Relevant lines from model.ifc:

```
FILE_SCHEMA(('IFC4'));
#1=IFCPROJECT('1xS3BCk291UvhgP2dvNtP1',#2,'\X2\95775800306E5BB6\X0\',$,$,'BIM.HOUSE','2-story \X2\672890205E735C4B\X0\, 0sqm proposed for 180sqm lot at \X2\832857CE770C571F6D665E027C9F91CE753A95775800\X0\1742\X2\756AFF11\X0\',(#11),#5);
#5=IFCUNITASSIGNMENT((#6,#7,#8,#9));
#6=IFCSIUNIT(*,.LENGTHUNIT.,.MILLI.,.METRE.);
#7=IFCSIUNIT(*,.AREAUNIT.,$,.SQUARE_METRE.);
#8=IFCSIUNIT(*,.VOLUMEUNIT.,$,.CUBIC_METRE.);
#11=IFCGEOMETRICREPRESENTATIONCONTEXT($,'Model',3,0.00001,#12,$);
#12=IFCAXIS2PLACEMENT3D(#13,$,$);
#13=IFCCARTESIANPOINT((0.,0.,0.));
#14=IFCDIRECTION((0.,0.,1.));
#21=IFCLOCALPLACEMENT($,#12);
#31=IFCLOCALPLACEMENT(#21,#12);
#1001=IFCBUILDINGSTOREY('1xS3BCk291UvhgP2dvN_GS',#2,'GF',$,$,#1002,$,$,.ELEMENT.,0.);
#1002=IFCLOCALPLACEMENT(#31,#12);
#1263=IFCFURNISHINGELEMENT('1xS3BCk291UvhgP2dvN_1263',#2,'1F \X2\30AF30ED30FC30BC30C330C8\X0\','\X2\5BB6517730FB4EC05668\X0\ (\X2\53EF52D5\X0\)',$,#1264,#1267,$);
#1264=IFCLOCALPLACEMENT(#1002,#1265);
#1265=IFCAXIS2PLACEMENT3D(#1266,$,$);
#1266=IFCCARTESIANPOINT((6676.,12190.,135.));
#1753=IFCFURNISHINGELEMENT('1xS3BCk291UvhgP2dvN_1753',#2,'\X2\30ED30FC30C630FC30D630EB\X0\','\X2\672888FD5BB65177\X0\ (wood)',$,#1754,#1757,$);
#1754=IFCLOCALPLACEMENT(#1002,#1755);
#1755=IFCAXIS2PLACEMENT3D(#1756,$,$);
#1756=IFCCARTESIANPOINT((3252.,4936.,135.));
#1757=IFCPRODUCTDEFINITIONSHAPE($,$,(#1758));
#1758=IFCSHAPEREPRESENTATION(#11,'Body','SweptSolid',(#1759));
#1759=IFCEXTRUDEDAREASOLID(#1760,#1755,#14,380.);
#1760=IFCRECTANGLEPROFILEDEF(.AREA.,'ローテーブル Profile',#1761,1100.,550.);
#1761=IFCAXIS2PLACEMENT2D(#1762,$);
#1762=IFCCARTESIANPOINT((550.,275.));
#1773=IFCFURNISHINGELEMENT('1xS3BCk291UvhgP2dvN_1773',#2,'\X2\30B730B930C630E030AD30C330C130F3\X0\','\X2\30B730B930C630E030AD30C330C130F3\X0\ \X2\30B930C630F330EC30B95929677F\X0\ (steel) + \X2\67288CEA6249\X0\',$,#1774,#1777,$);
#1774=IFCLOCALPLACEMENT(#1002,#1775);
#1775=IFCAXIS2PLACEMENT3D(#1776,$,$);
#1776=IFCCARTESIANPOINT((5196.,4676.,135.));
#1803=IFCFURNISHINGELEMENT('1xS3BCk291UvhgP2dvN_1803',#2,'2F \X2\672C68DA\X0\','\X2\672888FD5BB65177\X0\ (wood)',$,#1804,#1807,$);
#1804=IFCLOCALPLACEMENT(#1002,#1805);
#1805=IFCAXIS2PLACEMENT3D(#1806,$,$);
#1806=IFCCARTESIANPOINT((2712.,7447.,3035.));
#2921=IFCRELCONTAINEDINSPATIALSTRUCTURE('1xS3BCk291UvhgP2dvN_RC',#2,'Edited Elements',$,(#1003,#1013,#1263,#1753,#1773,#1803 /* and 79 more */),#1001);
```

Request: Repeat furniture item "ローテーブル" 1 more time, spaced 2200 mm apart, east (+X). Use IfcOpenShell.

```python
import numpy as np
import ifcopenshell
import ifcopenshell.api.geometry
import ifcopenshell.api.root
import ifcopenshell.util.element
import ifcopenshell.util.placement

model = ifcopenshell.open("model.ifc")


def reuse_history(source, copy):
    """copy_class also copies each property set's owner history, people and application; keep the originals."""
    for rel in copy.IsDefinedBy:
        if rel.is_a("IfcRelDefinesByProperties") and (history := rel.RelatingPropertyDefinition.OwnerHistory):
            rel.RelatingPropertyDefinition.OwnerHistory = source.OwnerHistory
            ifcopenshell.util.element.remove_deep2(model, history)


source = model.by_guid("1xS3BCk291UvhgP2dvN_1753")
base = ifcopenshell.util.placement.get_local_placement(source.ObjectPlacement)
step = np.array([1.0, 0.0, 0.0]) * 2200.0

for i in range(1, 2):
    copy = ifcopenshell.api.root.copy_class(model, product=source)
    copy.Representation = ifcopenshell.util.element.copy_deep(
        model, source.Representation, exclude=["IfcGeometricRepresentationContext", "IfcRepresentationMap"]
    )
    reuse_history(source, copy)
    matrix = base.copy()
    matrix[:3, 3] += i * step
    print("added at", matrix[:3, 3].round(3) + 0.0)
    ifcopenshell.api.geometry.edit_object_placement(model, product=copy, matrix=matrix, is_si=False)

model.write("model_updated.ifc")
```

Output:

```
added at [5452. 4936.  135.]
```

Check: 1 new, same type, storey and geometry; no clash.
